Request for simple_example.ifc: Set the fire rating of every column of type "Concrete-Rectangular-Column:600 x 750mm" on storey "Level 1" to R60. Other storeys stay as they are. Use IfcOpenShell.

First a look at what the model holds.

```python
import ifcopenshell
import ifcopenshell.util.element

model = ifcopenshell.open("simple_example.ifc")
print(model.schema)
storey = next(s for s in model.by_type("IfcBuildingStorey") if s.Name == "Level 1")
columns = [e for e in ifcopenshell.util.element.get_decomposition(storey) if e.is_a("IfcColumn")]
seen = {}
for e in columns:
    element_type = ifcopenshell.util.element.get_type(e)
    key = (element_type.Name if element_type != e and element_type else None, ifcopenshell.util.element.get_pset(e, "Pset_ColumnCommon", "FireRating"))
    seen[key] = seen.get(key, 0) + 1
for (name, value), count in sorted(seen.items(), key=str):
    print(count, "x", name, "|", value)
```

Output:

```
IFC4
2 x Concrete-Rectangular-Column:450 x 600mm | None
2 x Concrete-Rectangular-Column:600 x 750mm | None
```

```python
import ifcopenshell
import ifcopenshell.api.pset
import ifcopenshell.util.element

model = ifcopenshell.open("simple_example.ifc")

storey = next(s for s in model.by_type("IfcBuildingStorey") if s.Name == "Level 1")
columns = [e for e in ifcopenshell.util.element.get_decomposition(storey) if e.is_a("IfcColumn")]

count = 0
for e in columns:
    element_type = ifcopenshell.util.element.get_type(e)
    if element_type in (None, e) or element_type.Name != "Concrete-Rectangular-Column:600 x 750mm":
        continue
    # add_pset returns the element's existing set when there is one.
    pset = ifcopenshell.api.pset.add_pset(model, product=e, name="Pset_ColumnCommon")
    ifcopenshell.api.pset.edit_pset(model, pset=pset, properties={"FireRating": "R60"})
    count += 1

print(count, "columns updated")

model.write("simple_example_updated.ifc")
```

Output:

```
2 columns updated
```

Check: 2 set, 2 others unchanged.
